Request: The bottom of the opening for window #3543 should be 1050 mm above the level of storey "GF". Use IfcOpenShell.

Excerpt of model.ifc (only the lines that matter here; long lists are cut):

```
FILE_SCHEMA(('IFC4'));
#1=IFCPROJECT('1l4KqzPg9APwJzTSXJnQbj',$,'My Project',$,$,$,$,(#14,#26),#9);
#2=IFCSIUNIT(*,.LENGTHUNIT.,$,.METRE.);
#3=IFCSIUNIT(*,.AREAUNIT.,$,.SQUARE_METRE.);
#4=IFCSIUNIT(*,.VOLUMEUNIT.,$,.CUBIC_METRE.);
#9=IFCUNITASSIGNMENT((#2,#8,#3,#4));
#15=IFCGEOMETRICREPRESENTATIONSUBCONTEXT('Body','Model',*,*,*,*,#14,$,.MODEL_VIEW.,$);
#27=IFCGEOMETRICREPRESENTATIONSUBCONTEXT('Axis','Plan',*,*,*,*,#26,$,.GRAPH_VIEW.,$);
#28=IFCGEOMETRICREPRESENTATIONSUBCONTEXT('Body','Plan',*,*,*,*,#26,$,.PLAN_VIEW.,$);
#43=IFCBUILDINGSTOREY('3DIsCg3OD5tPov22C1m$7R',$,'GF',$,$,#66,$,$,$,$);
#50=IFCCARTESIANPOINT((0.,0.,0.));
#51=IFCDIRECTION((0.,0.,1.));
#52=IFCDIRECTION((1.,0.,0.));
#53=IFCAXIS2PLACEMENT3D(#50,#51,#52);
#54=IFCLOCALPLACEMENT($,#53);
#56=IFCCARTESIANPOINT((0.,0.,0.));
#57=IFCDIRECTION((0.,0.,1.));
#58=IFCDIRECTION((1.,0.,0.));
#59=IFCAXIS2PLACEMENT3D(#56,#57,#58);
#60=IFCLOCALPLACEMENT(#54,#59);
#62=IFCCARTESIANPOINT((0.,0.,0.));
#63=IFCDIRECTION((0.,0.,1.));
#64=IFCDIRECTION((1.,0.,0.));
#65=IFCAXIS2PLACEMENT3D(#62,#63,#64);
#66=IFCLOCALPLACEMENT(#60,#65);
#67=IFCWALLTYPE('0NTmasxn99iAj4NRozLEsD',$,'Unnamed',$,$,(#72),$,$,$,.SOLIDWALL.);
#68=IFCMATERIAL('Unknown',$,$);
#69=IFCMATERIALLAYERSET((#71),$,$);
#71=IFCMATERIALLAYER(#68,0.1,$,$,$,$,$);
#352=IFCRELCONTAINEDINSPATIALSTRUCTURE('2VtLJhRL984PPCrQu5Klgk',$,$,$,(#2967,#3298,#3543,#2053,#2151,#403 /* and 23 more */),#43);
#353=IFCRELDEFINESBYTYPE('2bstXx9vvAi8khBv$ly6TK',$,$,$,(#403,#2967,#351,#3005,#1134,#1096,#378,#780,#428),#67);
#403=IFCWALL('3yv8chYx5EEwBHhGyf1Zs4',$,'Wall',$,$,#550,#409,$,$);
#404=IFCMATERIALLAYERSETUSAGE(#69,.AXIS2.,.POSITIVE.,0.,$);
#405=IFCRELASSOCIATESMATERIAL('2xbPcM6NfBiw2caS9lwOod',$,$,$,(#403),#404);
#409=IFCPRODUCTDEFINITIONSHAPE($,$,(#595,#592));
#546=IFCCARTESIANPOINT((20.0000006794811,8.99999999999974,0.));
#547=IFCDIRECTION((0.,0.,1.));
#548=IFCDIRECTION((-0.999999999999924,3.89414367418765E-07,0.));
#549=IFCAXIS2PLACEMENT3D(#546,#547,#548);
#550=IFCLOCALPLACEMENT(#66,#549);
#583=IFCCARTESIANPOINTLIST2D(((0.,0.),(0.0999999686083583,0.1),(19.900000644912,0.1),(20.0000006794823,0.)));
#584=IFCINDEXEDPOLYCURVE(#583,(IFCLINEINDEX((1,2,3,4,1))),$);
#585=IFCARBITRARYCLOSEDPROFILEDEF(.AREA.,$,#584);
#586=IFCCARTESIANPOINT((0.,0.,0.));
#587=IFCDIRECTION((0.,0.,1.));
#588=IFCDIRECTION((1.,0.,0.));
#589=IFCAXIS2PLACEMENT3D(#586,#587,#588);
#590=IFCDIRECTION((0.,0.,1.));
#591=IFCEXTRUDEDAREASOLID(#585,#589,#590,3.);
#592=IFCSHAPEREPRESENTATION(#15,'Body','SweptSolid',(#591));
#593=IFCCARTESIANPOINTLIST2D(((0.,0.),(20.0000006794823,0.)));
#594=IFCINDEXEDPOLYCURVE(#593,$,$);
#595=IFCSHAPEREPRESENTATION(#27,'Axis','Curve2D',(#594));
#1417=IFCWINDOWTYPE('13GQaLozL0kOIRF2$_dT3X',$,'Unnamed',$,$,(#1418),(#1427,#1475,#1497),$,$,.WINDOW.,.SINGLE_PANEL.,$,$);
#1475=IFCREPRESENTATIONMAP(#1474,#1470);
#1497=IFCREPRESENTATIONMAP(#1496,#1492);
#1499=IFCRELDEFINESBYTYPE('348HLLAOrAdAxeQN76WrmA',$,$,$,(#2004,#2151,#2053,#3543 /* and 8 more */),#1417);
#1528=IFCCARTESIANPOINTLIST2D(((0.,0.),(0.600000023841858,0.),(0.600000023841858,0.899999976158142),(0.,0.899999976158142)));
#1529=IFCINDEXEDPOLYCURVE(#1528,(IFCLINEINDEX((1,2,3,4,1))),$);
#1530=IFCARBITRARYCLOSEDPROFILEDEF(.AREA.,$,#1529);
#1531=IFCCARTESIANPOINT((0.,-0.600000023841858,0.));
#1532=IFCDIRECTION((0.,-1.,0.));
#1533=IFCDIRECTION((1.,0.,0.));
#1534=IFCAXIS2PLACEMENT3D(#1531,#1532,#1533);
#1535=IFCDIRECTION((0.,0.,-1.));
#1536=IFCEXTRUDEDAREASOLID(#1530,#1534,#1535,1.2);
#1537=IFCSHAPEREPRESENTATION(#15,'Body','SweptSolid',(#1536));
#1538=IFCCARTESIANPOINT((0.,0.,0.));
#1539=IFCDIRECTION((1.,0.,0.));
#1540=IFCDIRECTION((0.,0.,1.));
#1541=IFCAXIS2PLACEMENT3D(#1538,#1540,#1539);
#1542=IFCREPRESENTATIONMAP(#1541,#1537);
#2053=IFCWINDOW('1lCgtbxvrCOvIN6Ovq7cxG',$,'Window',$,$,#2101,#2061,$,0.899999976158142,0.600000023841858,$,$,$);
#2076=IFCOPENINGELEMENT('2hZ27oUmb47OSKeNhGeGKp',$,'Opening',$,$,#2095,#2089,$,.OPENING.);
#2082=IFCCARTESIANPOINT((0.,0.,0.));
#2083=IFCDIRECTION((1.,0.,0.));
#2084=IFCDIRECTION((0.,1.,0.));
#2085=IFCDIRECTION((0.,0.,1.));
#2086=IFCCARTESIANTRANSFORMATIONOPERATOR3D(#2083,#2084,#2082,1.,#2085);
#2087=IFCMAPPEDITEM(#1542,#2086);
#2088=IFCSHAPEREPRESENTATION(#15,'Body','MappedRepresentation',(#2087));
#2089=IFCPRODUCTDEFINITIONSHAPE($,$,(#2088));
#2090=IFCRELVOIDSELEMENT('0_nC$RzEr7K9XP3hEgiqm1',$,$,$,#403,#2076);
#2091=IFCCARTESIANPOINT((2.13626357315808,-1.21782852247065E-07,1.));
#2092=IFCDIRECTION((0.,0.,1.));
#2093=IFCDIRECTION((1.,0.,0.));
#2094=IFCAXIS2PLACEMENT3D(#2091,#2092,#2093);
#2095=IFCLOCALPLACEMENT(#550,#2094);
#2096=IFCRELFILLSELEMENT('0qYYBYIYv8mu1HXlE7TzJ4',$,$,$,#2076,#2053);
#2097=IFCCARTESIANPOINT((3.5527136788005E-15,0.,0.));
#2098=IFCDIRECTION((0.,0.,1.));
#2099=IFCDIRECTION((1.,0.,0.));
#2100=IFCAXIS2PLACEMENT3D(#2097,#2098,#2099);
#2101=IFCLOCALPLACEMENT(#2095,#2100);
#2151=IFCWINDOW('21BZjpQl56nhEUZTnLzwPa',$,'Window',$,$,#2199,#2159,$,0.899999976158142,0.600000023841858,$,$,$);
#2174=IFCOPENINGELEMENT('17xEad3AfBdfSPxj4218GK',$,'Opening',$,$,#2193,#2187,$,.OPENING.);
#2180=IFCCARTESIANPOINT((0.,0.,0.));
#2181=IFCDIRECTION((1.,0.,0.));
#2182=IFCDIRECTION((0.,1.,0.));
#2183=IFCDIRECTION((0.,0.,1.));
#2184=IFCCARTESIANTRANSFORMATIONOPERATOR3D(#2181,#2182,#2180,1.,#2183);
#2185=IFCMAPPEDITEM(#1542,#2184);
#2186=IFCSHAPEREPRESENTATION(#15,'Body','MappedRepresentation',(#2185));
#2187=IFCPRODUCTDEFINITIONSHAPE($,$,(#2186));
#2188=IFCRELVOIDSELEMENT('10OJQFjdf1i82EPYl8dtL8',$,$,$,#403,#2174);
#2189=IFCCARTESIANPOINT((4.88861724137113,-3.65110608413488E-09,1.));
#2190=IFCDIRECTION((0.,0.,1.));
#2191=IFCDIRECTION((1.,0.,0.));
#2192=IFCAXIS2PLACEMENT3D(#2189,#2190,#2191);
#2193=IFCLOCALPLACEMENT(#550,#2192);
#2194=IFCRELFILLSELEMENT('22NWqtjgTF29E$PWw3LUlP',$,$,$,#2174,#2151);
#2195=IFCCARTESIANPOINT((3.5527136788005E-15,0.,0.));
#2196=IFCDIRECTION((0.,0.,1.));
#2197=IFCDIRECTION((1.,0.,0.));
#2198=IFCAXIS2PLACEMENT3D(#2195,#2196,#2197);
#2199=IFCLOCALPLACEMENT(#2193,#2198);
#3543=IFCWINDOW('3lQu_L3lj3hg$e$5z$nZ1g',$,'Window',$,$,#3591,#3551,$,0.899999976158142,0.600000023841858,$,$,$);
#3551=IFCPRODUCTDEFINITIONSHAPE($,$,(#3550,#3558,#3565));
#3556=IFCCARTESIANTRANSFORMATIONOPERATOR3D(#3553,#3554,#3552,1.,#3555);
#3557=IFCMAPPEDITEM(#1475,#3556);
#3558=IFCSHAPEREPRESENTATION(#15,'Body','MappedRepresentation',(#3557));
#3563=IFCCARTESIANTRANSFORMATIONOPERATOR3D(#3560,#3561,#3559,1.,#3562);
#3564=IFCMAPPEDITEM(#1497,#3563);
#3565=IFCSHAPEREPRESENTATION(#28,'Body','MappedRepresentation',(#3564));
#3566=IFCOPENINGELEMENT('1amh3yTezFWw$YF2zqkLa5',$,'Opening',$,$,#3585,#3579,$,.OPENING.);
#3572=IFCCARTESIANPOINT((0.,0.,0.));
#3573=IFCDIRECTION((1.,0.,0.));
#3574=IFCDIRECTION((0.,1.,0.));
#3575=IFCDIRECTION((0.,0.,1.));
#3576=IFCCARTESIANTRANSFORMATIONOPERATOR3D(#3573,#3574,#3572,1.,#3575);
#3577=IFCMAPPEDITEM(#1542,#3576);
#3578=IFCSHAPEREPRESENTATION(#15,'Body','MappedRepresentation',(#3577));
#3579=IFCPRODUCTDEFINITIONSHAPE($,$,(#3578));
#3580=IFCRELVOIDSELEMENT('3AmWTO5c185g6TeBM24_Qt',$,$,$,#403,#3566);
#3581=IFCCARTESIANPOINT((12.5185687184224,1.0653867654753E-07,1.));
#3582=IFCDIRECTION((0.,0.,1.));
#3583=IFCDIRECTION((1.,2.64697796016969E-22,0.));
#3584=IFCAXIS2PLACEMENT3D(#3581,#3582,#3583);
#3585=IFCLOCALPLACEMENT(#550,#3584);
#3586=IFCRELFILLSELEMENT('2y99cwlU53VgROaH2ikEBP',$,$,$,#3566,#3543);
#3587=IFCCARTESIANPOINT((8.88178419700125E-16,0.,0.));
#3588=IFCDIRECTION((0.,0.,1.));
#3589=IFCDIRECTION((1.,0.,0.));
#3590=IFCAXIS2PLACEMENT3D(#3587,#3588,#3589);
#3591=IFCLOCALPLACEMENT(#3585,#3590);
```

```python
import numpy as np
import ifcopenshell
import ifcopenshell.api.geometry
import ifcopenshell.geom
import ifcopenshell.util.element
import ifcopenshell.util.placement
import ifcopenshell.util.shape
import ifcopenshell.util.unit

model = ifcopenshell.open("model.ifc")
unit_scale = ifcopenshell.util.unit.calculate_unit_scale(model)

window = model.by_guid("3lQu_L3lj3hg$e$5z$nZ1g")
opening = window.FillsVoids[0].RelatingOpeningElement
storey = ifcopenshell.util.element.get_container(window, ifc_class="IfcBuildingStorey")
level = ifcopenshell.util.placement.get_local_placement(storey.ObjectPlacement)[2, 3]

# The opening's origin need not be at the sill, so measure its lowest point.
shape = ifcopenshell.geom.create_shape(ifcopenshell.geom.settings(), opening)
bottom = ifcopenshell.util.shape.get_shape_bottom_elevation(shape, shape.geometry) / unit_scale
dz = level + 1.05 - bottom

shift = np.array([0.0, 0.0, dz])
# The window is placed relative to its opening, so it follows when the opening moves.
matrix = ifcopenshell.util.placement.get_local_placement(opening.ObjectPlacement)
matrix[:3, 3] += shift
ifcopenshell.api.geometry.edit_object_placement(
    model, product=opening, matrix=matrix, is_si=False, should_transform_children=True
)

print(f"moved by {dz * unit_scale:+.3f} m")

model.write("model_rev.ifc")
```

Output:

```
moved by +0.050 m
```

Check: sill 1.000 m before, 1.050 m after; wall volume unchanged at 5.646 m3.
